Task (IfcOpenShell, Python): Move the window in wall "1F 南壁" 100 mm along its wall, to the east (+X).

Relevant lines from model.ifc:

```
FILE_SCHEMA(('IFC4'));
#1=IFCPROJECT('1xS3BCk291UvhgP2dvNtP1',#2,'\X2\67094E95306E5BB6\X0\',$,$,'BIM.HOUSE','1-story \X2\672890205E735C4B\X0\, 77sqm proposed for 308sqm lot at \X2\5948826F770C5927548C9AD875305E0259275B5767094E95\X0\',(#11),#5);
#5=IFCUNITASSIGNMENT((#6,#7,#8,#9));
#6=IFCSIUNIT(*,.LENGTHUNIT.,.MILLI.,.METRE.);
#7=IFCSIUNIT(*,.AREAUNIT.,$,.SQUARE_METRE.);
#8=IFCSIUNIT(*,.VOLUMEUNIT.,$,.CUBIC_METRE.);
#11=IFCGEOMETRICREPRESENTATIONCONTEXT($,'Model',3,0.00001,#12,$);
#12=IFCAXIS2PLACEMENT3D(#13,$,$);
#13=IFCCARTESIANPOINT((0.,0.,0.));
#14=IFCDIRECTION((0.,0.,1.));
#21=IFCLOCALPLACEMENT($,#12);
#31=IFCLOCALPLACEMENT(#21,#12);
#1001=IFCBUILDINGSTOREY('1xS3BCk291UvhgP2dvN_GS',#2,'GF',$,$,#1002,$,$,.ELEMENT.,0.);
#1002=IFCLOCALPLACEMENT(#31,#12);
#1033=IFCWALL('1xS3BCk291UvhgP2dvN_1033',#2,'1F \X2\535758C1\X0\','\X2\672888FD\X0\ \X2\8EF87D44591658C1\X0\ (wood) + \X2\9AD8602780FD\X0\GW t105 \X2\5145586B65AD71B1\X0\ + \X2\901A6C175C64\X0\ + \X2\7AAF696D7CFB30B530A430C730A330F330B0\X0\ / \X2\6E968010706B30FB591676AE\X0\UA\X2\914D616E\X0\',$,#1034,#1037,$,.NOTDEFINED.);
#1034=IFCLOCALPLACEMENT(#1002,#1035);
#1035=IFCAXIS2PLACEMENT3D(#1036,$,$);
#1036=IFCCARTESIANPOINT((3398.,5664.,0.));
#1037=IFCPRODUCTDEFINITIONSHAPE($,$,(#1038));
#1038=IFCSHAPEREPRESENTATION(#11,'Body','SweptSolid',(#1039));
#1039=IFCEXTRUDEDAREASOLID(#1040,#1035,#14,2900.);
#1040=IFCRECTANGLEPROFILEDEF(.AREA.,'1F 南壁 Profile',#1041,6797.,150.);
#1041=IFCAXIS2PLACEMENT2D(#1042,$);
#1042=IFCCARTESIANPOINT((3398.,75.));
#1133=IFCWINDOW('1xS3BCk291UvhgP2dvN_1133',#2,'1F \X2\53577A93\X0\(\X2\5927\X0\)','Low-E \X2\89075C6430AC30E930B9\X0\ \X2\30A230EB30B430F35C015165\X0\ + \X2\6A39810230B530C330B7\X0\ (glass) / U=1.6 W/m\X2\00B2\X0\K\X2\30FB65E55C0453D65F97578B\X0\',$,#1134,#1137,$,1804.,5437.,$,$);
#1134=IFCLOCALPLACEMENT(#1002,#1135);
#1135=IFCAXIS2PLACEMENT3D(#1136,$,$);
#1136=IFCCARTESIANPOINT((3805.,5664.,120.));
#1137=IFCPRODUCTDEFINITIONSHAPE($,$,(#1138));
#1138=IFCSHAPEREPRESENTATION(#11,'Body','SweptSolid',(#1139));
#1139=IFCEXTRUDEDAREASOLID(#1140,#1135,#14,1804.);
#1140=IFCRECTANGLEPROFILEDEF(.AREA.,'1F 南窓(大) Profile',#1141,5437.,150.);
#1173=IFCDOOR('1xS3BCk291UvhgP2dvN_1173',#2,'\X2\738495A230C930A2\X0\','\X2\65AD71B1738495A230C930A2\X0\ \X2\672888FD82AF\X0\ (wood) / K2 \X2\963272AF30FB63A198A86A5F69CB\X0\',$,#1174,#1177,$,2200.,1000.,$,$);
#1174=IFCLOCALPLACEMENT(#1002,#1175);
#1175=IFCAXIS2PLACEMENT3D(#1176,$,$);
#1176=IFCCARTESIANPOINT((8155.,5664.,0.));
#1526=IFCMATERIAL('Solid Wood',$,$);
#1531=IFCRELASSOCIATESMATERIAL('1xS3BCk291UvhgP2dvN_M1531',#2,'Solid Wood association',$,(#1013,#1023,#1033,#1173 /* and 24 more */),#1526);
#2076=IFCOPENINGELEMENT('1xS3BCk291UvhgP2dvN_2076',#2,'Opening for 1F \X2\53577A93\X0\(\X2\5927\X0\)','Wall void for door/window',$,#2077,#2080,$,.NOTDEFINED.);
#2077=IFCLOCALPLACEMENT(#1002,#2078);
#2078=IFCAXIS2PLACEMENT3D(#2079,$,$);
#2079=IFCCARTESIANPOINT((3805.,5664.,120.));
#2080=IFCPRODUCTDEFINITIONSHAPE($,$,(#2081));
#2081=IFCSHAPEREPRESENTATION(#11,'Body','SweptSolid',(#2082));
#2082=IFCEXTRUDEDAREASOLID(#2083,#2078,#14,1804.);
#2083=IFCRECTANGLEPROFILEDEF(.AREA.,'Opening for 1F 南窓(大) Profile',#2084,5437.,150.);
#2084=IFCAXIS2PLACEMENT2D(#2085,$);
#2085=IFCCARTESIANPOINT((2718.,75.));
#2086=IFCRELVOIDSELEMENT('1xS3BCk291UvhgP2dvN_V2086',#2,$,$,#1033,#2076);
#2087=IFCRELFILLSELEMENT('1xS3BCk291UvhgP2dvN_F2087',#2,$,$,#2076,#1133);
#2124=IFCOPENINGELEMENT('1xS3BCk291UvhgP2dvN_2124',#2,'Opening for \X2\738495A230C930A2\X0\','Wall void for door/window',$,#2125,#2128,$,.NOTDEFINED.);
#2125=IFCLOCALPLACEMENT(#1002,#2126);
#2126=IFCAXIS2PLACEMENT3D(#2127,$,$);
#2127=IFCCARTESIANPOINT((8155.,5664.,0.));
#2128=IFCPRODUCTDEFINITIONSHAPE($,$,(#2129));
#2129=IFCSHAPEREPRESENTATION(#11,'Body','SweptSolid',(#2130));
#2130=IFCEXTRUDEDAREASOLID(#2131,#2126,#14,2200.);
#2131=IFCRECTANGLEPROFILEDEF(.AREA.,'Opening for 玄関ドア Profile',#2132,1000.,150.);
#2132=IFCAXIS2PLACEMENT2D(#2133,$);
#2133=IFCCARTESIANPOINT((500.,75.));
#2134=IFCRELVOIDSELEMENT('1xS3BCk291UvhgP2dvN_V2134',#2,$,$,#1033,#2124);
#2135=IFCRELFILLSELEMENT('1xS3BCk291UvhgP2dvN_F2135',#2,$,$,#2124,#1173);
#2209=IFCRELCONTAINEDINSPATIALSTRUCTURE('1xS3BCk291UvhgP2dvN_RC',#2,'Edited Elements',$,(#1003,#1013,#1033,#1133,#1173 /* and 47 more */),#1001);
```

```python
import ifcopenshell
import ifcopenshell.api.geometry
import ifcopenshell.util.placement
import ifcopenshell.util.unit

model = ifcopenshell.open("model.ifc")
unit_scale = ifcopenshell.util.unit.calculate_unit_scale(model)

window = model.by_guid("1xS3BCk291UvhgP2dvN_1133")
opening = window.FillsVoids[0].RelatingOpeningElement
wall = opening.VoidsElements[0].RelatingBuildingElement

wall_matrix = ifcopenshell.util.placement.get_local_placement(wall.ObjectPlacement)
shift = wall_matrix[:3, 0] * 0.1 / unit_scale
before = ifcopenshell.util.placement.get_local_placement(window.ObjectPlacement)[:3, 3].copy()

# The window is not placed relative to its opening, so move both.
for product in (opening, window):
    matrix = ifcopenshell.util.placement.get_local_placement(product.ObjectPlacement)
    matrix[:3, 3] += shift
    ifcopenshell.api.geometry.edit_object_placement(model, product=product, matrix=matrix, is_si=False)

after = ifcopenshell.util.placement.get_local_placement(window.ObjectPlacement)[:3, 3]
print("window moved by", (after - before).round(3) + 0.0)

model.write("model_v2.ifc")
```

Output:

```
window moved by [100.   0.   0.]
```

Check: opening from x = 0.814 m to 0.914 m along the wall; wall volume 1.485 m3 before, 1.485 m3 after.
